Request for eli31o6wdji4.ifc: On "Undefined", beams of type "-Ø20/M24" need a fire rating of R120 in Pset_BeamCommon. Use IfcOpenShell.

First a look at what the model holds.

```python
import ifcopenshell
import ifcopenshell.util.element

model = ifcopenshell.open("eli31o6wdji4.ifc")
print(model.schema)
storey = next(s for s in model.by_type("IfcBuildingStorey") if s.Name == "Undefined")
beams = [e for e in ifcopenshell.util.element.get_decomposition(storey) if e.is_a("IfcBeam")]
seen = {}
for e in beams:
    element_type = ifcopenshell.util.element.get_type(e)
    key = (element_type.Name if element_type != e and element_type else None, ifcopenshell.util.element.get_pset(e, "Pset_BeamCommon", "FireRating"))
    seen[key] = seen.get(key, 0) + 1
for (name, value), count in sorted(seen.items(), key=str):
    print(count, "x", name, "|", value)
```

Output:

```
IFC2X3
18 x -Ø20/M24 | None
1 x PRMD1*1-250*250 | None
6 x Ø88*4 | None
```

```python
import ifcopenshell
import ifcopenshell.api.pset
import ifcopenshell.util.element

model = ifcopenshell.open("eli31o6wdji4.ifc")

storey = next(s for s in model.by_type("IfcBuildingStorey") if s.Name == "Undefined")
beams = [e for e in ifcopenshell.util.element.get_decomposition(storey) if e.is_a("IfcBeam")]

count = 0
for e in beams:
    element_type = ifcopenshell.util.element.get_type(e)
    if element_type in (None, e) or element_type.Name != "-Ø20/M24":
        continue
    found = ifcopenshell.util.element.get_pset(e, "Pset_BeamCommon", should_inherit=False)
    if found:
        pset = model.by_id(found["id"])
        if len(ifcopenshell.util.element.get_elements_by_pset(pset)) > 1:
            pset = ifcopenshell.api.pset.unshare_pset(model, products=[e], pset=pset)[0]
    else:
        pset = ifcopenshell.api.pset.add_pset(model, product=e, name="Pset_BeamCommon")
    ifcopenshell.api.pset.edit_pset(model, pset=pset, properties={"FireRating": "R120"})
    count += 1

print(count, "beams updated")

model.write("eli31o6wdji4_updated.ifc")
```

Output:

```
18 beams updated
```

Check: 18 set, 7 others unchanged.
